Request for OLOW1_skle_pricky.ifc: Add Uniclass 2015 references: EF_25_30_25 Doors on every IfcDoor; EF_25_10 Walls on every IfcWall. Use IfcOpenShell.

First a look at what the model holds.

```python
import ifcopenshell

model = ifcopenshell.open("OLOW1_skle_pricky.ifc")
print(model.schema)
print("classifications:", [c.Name for c in model.by_type("IfcClassification")])
for ifc_class in ("IfcDoor", "IfcRoof", "IfcStair", "IfcWall", "IfcWindow"):
    print(ifc_class, len(model.by_type(ifc_class)))
```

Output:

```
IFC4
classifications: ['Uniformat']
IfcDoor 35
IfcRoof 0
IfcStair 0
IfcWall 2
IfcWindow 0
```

```python
import ifcopenshell
import ifcopenshell.api.classification

model = ifcopenshell.open("OLOW1_skle_pricky.ifc")

system = ifcopenshell.api.classification.add_classification(model, classification="Uniclass 2015")

codes = {
    "IfcDoor": ("EF_25_30_25", "Doors"),
    "IfcWall": ("EF_25_10", "Walls"),
}
for ifc_class, (code, name) in codes.items():
    products = model.by_type(ifc_class)
    ifcopenshell.api.classification.add_reference(
        model, products=products, classification=system, identification=code, name=name
    )
    print(code, len(products))

model.write("OLOW1_skle_pricky_v2.ifc")
```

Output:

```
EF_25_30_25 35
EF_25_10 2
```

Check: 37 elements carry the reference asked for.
